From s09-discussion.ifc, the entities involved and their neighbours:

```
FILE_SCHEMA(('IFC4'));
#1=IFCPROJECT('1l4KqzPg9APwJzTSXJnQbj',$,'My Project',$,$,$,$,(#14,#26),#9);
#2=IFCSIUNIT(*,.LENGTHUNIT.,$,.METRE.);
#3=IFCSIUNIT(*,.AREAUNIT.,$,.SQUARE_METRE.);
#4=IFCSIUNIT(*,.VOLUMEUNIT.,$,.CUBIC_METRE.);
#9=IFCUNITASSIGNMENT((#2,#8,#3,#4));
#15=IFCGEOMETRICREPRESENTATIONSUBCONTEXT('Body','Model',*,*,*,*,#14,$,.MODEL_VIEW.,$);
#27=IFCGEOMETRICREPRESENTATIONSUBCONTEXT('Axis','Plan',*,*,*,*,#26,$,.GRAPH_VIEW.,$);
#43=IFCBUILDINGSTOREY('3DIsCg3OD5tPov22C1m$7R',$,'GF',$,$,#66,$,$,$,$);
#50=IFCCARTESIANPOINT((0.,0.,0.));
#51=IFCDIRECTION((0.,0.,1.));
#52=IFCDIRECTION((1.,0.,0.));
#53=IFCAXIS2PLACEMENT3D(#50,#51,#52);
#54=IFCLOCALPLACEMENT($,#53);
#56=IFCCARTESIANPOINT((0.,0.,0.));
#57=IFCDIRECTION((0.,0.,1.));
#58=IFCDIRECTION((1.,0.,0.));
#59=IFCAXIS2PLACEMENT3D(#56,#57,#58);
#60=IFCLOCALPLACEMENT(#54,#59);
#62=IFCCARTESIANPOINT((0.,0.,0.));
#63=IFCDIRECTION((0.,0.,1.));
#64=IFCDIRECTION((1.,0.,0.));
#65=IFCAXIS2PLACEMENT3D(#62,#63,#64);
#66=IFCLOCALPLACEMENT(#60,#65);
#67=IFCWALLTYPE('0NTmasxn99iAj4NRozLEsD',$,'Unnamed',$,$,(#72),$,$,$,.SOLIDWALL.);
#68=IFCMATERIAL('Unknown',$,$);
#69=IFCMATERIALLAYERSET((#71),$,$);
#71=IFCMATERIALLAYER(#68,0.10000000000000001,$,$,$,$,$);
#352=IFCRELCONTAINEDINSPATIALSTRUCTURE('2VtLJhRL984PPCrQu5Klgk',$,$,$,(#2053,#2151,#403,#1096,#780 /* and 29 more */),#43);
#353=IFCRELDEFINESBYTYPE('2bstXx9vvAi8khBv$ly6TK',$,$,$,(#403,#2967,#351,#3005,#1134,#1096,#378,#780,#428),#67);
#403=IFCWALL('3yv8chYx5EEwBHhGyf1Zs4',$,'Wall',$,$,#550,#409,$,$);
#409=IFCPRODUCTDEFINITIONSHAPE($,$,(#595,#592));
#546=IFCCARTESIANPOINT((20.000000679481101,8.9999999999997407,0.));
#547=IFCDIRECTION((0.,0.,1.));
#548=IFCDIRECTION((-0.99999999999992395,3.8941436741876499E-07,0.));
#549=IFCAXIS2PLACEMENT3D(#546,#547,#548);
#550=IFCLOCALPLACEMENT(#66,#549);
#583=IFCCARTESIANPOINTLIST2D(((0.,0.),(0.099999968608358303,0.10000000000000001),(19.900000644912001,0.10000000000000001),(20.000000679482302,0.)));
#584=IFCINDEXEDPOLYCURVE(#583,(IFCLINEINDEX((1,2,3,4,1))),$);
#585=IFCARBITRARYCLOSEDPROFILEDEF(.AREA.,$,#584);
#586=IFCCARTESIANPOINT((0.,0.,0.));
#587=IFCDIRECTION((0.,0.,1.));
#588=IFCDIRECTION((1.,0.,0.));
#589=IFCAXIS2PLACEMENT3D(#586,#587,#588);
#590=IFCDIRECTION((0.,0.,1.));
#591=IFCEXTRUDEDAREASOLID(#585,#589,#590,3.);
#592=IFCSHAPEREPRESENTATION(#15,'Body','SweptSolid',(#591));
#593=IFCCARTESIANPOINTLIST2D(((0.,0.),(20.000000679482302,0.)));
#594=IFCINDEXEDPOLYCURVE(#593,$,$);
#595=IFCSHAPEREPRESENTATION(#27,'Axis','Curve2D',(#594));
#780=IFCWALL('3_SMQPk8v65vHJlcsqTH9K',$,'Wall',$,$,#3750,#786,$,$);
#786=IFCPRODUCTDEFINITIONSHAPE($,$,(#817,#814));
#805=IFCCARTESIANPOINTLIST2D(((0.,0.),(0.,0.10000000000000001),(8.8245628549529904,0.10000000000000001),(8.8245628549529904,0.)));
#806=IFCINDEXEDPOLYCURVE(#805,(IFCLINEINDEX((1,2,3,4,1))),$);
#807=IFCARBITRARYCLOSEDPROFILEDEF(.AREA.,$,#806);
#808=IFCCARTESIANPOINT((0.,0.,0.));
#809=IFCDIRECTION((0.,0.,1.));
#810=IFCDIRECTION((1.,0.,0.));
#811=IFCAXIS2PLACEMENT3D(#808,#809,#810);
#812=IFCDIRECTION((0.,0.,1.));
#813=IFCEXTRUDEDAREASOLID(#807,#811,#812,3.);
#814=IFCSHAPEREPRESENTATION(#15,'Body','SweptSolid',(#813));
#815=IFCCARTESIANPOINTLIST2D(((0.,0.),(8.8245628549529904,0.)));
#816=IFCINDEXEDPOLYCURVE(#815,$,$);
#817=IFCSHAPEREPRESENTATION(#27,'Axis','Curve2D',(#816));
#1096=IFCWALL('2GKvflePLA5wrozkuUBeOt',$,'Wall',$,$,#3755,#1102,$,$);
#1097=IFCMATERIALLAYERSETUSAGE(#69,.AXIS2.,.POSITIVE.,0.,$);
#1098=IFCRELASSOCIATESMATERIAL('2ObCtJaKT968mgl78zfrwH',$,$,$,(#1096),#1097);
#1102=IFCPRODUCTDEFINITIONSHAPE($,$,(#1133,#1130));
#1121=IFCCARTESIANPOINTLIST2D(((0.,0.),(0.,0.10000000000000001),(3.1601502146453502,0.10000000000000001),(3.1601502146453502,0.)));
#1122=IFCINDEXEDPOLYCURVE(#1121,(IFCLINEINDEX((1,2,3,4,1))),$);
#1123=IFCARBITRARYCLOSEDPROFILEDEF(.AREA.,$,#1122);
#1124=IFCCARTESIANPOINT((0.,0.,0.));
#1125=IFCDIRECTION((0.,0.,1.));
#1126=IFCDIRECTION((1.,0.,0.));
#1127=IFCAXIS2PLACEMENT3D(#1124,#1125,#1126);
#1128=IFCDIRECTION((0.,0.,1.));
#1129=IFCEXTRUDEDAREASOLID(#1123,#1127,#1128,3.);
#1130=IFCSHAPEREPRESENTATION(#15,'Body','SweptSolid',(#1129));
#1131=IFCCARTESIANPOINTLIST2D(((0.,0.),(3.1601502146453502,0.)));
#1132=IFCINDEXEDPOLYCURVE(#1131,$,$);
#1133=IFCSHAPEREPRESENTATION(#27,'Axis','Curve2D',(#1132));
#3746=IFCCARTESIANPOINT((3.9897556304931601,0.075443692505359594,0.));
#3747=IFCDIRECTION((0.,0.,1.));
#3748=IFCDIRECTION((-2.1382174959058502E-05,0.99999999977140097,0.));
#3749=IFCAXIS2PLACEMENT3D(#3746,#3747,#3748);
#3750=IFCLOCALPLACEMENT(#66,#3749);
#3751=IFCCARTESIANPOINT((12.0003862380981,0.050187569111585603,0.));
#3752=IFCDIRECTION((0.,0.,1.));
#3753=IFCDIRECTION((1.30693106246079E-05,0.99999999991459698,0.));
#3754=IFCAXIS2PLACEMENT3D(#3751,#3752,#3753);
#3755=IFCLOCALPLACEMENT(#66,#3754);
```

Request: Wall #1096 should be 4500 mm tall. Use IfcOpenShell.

```python
import ifcopenshell
import ifcopenshell.geom
import ifcopenshell.util.representation
import ifcopenshell.util.shape

model = ifcopenshell.open("s09-discussion.ifc")
settings = ifcopenshell.geom.settings()


def volume(element):
    """Net volume in cubic metres, openings subtracted."""
    shape = ifcopenshell.geom.create_shape(settings, element)
    return ifcopenshell.util.shape.get_volume(shape.geometry)


wall = model.by_guid("2GKvflePLA5wrozkuUBeOt")
before = volume(wall)

body = ifcopenshell.util.representation.get_representation(wall, "Model", "Body")
solid = body.Items[0]
old_height = solid.Depth
solid.Depth = 4.5
after = volume(wall)

print(f"height {old_height:g} -> {solid.Depth:g}, volume {before:.3f} -> {after:.3f} m3")

model.write("s09-discussion-out.ifc")
```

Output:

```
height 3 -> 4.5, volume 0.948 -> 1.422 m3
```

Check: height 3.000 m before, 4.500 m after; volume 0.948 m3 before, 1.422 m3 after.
